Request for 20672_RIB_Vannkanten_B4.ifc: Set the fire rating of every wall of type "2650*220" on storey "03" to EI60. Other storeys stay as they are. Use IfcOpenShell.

First a look at what the model holds.

```python
import ifcopenshell
import ifcopenshell.util.element

model = ifcopenshell.open("20672_RIB_Vannkanten_B4.ifc")
print(model.schema)
storey = next(s for s in model.by_type("IfcBuildingStorey") if s.Name == "03")
walls = [e for e in ifcopenshell.util.element.get_decomposition(storey) if e.is_a("IfcWall")]
seen = {}
for e in walls:
    element_type = ifcopenshell.util.element.get_type(e)
    key = (element_type.Name if element_type != e and element_type else None, ifcopenshell.util.element.get_pset(e, "Pset_WallCommon", "FireRating"))
    seen[key] = seen.get(key, 0) + 1
for (name, value), count in sorted(seen.items(), key=str):
    print(count, "x", name, "|", value)
```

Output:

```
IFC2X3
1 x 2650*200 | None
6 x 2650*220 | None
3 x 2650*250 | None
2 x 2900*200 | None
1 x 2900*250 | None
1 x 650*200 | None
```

```python
import ifcopenshell
import ifcopenshell.api.pset
import ifcopenshell.util.element

model = ifcopenshell.open("20672_RIB_Vannkanten_B4.ifc")

storey = next(s for s in model.by_type("IfcBuildingStorey") if s.Name == "03")
walls = [e for e in ifcopenshell.util.element.get_decomposition(storey) if e.is_a("IfcWall")]

count = 0
for e in walls:
    element_type = ifcopenshell.util.element.get_type(e)
    if element_type in (None, e) or element_type.Name != "2650*220":
        continue
    # add_pset returns the element's existing set when there is one.
    pset = ifcopenshell.api.pset.add_pset(model, product=e, name="Pset_WallCommon")
    ifcopenshell.api.pset.edit_pset(model, pset=pset, properties={"FireRating": "EI60"})
    count += 1

print(count, "walls updated")

model.write("20672_RIB_Vannkanten_B4-out.ifc")
```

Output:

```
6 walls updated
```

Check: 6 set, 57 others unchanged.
